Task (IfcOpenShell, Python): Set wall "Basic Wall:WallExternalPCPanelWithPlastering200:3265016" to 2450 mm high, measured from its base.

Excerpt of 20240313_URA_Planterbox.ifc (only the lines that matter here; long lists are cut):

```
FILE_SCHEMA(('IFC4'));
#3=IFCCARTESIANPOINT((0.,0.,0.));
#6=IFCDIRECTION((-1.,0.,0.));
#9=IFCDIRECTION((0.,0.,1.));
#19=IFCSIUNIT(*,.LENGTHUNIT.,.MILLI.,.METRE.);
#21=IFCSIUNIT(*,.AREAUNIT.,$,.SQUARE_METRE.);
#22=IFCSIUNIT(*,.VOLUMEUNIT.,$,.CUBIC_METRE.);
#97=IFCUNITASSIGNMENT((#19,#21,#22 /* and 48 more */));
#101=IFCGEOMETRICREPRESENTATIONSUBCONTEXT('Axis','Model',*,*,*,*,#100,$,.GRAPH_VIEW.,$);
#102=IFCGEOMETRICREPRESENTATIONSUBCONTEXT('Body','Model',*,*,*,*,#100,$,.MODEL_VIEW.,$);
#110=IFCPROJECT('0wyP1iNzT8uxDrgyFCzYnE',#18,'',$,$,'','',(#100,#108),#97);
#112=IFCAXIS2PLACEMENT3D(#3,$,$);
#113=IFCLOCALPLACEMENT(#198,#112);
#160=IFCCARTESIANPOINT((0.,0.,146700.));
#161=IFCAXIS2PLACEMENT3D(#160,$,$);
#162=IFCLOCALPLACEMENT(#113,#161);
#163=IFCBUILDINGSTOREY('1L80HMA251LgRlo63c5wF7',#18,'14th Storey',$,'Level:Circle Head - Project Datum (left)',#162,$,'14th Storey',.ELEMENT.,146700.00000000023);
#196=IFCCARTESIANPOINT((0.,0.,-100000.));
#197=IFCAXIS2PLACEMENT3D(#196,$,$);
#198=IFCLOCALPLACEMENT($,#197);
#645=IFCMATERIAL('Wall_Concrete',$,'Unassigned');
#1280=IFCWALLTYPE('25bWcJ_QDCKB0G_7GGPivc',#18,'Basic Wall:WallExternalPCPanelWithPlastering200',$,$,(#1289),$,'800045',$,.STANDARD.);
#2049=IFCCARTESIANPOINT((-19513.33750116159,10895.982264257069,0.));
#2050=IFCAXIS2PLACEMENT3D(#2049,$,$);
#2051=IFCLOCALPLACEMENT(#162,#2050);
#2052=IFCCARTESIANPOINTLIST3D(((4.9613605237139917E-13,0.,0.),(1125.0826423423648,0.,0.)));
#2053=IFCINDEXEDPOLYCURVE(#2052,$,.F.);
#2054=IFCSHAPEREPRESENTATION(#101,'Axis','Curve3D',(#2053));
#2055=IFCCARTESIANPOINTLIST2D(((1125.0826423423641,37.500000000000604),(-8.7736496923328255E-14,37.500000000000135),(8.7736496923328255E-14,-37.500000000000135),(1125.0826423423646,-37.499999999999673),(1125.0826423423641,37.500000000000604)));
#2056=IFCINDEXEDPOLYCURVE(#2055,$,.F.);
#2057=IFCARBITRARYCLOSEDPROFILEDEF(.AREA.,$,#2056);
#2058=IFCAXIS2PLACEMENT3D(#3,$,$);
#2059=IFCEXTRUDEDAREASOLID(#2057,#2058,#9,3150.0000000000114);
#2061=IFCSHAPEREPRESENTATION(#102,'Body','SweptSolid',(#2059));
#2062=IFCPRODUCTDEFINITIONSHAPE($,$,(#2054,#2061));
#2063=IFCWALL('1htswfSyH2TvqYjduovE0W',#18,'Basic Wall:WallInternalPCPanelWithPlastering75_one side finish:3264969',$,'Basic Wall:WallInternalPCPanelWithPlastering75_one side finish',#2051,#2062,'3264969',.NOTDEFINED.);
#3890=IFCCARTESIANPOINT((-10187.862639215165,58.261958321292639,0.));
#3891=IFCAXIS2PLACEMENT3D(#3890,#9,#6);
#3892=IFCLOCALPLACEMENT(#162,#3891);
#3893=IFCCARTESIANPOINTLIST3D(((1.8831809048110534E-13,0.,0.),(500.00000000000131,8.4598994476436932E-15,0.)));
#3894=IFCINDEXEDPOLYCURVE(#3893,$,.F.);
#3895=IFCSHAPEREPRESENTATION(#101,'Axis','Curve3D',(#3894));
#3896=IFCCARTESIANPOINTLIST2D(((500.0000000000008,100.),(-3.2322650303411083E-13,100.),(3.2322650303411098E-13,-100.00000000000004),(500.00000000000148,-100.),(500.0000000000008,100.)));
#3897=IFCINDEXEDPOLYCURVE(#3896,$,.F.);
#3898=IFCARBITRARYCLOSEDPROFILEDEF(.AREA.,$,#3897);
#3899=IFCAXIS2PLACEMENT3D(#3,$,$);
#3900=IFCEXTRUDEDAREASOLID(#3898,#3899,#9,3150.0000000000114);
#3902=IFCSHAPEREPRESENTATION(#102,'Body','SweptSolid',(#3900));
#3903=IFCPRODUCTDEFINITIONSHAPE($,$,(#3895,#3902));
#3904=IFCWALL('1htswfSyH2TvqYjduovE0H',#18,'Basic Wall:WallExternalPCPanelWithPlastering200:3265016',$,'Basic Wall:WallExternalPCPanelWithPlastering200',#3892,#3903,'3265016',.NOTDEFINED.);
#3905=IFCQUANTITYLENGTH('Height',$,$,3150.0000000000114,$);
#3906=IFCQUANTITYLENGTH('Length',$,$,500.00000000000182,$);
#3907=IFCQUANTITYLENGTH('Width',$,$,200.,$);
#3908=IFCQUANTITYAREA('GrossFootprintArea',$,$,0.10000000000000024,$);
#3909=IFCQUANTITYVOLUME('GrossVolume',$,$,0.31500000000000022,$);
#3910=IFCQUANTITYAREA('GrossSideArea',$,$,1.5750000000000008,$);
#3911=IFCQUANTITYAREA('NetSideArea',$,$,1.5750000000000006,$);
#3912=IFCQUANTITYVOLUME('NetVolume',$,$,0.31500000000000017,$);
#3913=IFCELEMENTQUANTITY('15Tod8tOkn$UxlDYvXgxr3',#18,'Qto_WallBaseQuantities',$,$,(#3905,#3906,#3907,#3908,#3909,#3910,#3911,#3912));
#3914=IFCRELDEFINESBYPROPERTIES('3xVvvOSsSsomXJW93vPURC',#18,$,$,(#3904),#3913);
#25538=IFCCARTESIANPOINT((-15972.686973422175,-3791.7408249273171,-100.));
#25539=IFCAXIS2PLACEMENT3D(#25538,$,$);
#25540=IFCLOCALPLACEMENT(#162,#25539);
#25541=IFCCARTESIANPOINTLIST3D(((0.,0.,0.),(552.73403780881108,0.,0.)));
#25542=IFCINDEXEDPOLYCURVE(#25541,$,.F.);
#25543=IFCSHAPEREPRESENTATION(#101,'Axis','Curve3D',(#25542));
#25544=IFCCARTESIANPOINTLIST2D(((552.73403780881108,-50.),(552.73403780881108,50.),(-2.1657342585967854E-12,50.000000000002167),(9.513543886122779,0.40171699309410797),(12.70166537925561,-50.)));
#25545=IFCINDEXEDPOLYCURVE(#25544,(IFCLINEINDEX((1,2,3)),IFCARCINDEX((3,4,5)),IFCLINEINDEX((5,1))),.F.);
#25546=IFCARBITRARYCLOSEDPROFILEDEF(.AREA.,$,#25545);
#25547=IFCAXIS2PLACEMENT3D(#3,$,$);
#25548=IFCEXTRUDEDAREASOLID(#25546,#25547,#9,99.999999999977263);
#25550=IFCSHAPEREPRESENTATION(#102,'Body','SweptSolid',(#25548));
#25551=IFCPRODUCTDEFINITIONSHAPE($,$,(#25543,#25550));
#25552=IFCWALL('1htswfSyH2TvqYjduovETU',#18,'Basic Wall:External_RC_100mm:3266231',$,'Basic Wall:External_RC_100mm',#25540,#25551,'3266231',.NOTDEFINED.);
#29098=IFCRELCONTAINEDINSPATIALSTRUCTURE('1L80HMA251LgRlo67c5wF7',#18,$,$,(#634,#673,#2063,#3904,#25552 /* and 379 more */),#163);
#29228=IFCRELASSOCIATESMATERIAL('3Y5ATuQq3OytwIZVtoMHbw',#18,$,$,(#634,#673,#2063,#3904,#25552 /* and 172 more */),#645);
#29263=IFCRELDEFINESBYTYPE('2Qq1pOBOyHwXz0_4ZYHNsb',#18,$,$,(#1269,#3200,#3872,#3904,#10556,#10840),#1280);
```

```python
import ifcopenshell
import ifcopenshell.api.pset
import ifcopenshell.geom
import ifcopenshell.util.element
import ifcopenshell.util.representation
import ifcopenshell.util.shape
import ifcopenshell.util.unit

model = ifcopenshell.open("20240313_URA_Planterbox.ifc")
unit_scale = ifcopenshell.util.unit.calculate_unit_scale(model)
area_scale = ifcopenshell.util.unit.calculate_unit_scale(model, "AREAUNIT")
volume_scale = ifcopenshell.util.unit.calculate_unit_scale(model, "VOLUMEUNIT")
settings = ifcopenshell.geom.settings()


def volume(element):
    """Net volume in cubic metres, openings subtracted."""
    shape = ifcopenshell.geom.create_shape(settings, element)
    return ifcopenshell.util.shape.get_volume(shape.geometry)


wall = model.by_guid("1htswfSyH2TvqYjduovE0H")
before = volume(wall)

body = ifcopenshell.util.representation.get_representation(wall, "Model", "Body")
solid = body.Items[0]
old_height = solid.Depth
solid.Depth = 2450.0
after = volume(wall)
thickness = 0.2  # wall thickness in metres

# Update the stored height, areas and volumes.
qto = model.by_id(ifcopenshell.util.element.get_pset(wall, "Qto_WallBaseQuantities", should_inherit=False)["id"])
ifcopenshell.api.pset.edit_qto(model, qto=qto, properties={
    "Height": solid.Depth,
    "GrossVolume": ifcopenshell.util.element.get_pset(wall, "Qto_WallBaseQuantities", "GrossVolume") * solid.Depth / old_height,
    "GrossSideArea": ifcopenshell.util.element.get_pset(wall, "Qto_WallBaseQuantities", "GrossSideArea") * solid.Depth / old_height,
    "NetSideArea": after / thickness / area_scale,
    "NetVolume": after / volume_scale,
})

print(f"height {old_height:g} -> {solid.Depth:g}, volume {before:.3f} -> {after:.3f} m3")

model.write("20240313_URA_Planterbox_v2.ifc")
```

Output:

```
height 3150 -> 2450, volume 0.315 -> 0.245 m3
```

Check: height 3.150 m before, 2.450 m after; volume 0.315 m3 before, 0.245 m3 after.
